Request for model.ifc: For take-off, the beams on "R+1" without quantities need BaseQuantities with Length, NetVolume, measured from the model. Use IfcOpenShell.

First a look at what the model holds.

```python
import ifcopenshell
import ifcopenshell.util.element
import ifcopenshell.util.unit

model = ifcopenshell.open("model.ifc")
print(model.schema)
for unit_type in ("LENGTHUNIT", "AREAUNIT", "VOLUMEUNIT"):
    print(unit_type, ifcopenshell.util.unit.calculate_unit_scale(model, unit_type))
storey = next(s for s in model.by_type("IfcBuildingStorey") if s.Name == "R+1")
beams = [e for e in ifcopenshell.util.element.get_decomposition(storey) if e.is_a("IfcBeam")]
for e in sorted(beams, key=lambda e: e.id()):
    print(e.id(), e.is_a(), e.Name, list(ifcopenshell.util.element.get_psets(e, qtos_only=True)), sep=" | ")
```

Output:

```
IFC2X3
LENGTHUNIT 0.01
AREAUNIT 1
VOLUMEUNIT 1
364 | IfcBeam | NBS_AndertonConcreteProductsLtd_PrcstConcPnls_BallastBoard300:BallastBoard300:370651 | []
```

```python
import ifcopenshell
import ifcopenshell.api.pset
import ifcopenshell.geom
import ifcopenshell.util.element
import ifcopenshell.util.shape
import ifcopenshell.util.unit

model = ifcopenshell.open("model.ifc")
unit_scale = ifcopenshell.util.unit.calculate_unit_scale(model)
volume_scale = ifcopenshell.util.unit.calculate_unit_scale(model, "VOLUMEUNIT")
settings = ifcopenshell.geom.settings()

storey = next(s for s in model.by_type("IfcBuildingStorey") if s.Name == "R+1")
beams = [e for e in ifcopenshell.util.element.get_decomposition(storey) if e.is_a("IfcBeam")]

for e in sorted(beams, key=lambda e: e.id()):
    if ifcopenshell.util.element.get_psets(e, qtos_only=True, should_inherit=False):
        continue
    # Geometry comes back in metres, in the element's own axes.
    shape = ifcopenshell.geom.create_shape(settings, e)
    values = {
        "Length": ifcopenshell.util.shape.get_max_xyz(shape.geometry) / unit_scale,
        "NetVolume": ifcopenshell.util.shape.get_volume(shape.geometry) / volume_scale,
    }
    qto = ifcopenshell.api.pset.add_qto(model, product=e, name="BaseQuantities")
    ifcopenshell.api.pset.edit_qto(model, qto=qto, properties=values)
    print(e.id(), {k: round(v, 3) for k, v in values.items()})

model.write("model_rev.ifc")
```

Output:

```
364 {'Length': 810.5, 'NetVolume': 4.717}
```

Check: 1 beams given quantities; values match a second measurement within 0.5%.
